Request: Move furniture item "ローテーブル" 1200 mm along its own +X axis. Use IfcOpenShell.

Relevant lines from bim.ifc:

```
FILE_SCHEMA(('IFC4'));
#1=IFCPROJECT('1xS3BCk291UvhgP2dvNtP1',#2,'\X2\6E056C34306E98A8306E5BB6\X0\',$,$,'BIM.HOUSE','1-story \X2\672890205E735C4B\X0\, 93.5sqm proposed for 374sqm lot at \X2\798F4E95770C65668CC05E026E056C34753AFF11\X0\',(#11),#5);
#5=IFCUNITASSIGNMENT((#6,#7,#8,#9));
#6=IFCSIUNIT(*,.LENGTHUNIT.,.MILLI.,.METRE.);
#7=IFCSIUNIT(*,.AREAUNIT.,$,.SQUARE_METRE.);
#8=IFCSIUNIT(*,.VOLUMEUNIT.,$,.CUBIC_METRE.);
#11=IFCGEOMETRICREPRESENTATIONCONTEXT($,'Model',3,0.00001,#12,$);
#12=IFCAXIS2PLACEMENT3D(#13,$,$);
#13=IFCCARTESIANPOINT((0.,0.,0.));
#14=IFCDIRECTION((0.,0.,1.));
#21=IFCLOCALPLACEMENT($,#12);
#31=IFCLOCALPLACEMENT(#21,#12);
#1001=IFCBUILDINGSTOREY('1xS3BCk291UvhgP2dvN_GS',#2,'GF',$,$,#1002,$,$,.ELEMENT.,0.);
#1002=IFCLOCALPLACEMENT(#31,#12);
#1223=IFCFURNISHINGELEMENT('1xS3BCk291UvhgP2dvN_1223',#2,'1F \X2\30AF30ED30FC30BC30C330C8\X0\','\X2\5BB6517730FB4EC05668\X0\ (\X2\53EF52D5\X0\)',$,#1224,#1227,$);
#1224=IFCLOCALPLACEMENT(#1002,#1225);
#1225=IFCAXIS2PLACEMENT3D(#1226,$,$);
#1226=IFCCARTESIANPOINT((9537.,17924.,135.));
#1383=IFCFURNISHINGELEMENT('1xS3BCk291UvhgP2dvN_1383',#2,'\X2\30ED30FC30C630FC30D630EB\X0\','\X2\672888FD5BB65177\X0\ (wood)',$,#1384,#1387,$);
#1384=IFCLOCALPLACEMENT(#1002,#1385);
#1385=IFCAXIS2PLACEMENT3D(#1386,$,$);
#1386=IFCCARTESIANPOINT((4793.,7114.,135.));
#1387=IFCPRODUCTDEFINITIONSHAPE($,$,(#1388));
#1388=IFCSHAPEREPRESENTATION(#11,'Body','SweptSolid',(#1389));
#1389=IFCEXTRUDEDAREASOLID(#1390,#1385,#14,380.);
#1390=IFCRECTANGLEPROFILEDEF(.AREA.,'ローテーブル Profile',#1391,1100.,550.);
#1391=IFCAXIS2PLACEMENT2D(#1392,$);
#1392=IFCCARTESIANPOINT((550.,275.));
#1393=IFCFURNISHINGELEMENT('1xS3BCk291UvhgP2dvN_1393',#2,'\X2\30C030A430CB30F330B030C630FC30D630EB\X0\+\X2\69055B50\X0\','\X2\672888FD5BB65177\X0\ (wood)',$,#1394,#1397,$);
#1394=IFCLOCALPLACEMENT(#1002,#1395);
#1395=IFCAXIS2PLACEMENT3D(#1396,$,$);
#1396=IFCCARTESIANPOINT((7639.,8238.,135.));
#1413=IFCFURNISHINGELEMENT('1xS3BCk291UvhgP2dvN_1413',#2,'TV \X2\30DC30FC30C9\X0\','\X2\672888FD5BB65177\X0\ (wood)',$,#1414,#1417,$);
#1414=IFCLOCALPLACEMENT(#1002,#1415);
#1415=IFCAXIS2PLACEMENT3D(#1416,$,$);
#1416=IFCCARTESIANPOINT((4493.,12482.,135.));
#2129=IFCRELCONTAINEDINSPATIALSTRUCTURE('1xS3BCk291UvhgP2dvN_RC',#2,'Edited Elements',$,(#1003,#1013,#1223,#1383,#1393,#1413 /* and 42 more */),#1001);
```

```python
import ifcopenshell
import ifcopenshell.api.geometry
import ifcopenshell.util.placement
import ifcopenshell.util.unit

model = ifcopenshell.open("bim.ifc")
unit_scale = ifcopenshell.util.unit.calculate_unit_scale(model)

item = model.by_id(1383)
matrix = ifcopenshell.util.placement.get_local_placement(item.ObjectPlacement)
matrix[:3, 3] += matrix[:3, 0] * 1.2 / unit_scale
ifcopenshell.api.geometry.edit_object_placement(model, product=item, matrix=matrix, is_si=False)

print(ifcopenshell.util.placement.get_local_placement(item.ObjectPlacement).round(3) + 0.0)

model.write("bim_edited.ifc")
```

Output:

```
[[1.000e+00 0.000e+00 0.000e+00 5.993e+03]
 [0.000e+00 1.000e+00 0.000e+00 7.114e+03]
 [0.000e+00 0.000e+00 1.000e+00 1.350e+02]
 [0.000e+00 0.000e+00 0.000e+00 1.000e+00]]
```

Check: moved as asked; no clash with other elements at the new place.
